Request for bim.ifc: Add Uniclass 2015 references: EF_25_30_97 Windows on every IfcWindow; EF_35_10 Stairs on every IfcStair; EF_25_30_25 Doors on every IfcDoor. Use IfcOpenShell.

First a look at what the model holds.

```python
import ifcopenshell

model = ifcopenshell.open("bim.ifc")
print(model.schema)
print("classifications:", [c.Name for c in model.by_type("IfcClassification")])
for ifc_class in ("IfcDoor", "IfcRoof", "IfcStair", "IfcWall", "IfcWindow"):
    print(ifc_class, len(model.by_type(ifc_class)))
```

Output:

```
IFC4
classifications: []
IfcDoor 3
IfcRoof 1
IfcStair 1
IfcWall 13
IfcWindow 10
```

```python
import ifcopenshell
import ifcopenshell.api.classification

model = ifcopenshell.open("bim.ifc")

system = ifcopenshell.api.classification.add_classification(model, classification="Uniclass 2015")

codes = {
    "IfcWindow": ("EF_25_30_97", "Windows"),
    "IfcStair": ("EF_35_10", "Stairs"),
    "IfcDoor": ("EF_25_30_25", "Doors"),
}
for ifc_class, (code, name) in codes.items():
    products = model.by_type(ifc_class)
    ifcopenshell.api.classification.add_reference(
        model, products=products, classification=system, identification=code, name=name
    )
    print(code, len(products))

model.write("bim_updated.ifc")
```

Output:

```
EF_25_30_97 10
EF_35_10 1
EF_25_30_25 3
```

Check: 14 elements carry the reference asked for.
